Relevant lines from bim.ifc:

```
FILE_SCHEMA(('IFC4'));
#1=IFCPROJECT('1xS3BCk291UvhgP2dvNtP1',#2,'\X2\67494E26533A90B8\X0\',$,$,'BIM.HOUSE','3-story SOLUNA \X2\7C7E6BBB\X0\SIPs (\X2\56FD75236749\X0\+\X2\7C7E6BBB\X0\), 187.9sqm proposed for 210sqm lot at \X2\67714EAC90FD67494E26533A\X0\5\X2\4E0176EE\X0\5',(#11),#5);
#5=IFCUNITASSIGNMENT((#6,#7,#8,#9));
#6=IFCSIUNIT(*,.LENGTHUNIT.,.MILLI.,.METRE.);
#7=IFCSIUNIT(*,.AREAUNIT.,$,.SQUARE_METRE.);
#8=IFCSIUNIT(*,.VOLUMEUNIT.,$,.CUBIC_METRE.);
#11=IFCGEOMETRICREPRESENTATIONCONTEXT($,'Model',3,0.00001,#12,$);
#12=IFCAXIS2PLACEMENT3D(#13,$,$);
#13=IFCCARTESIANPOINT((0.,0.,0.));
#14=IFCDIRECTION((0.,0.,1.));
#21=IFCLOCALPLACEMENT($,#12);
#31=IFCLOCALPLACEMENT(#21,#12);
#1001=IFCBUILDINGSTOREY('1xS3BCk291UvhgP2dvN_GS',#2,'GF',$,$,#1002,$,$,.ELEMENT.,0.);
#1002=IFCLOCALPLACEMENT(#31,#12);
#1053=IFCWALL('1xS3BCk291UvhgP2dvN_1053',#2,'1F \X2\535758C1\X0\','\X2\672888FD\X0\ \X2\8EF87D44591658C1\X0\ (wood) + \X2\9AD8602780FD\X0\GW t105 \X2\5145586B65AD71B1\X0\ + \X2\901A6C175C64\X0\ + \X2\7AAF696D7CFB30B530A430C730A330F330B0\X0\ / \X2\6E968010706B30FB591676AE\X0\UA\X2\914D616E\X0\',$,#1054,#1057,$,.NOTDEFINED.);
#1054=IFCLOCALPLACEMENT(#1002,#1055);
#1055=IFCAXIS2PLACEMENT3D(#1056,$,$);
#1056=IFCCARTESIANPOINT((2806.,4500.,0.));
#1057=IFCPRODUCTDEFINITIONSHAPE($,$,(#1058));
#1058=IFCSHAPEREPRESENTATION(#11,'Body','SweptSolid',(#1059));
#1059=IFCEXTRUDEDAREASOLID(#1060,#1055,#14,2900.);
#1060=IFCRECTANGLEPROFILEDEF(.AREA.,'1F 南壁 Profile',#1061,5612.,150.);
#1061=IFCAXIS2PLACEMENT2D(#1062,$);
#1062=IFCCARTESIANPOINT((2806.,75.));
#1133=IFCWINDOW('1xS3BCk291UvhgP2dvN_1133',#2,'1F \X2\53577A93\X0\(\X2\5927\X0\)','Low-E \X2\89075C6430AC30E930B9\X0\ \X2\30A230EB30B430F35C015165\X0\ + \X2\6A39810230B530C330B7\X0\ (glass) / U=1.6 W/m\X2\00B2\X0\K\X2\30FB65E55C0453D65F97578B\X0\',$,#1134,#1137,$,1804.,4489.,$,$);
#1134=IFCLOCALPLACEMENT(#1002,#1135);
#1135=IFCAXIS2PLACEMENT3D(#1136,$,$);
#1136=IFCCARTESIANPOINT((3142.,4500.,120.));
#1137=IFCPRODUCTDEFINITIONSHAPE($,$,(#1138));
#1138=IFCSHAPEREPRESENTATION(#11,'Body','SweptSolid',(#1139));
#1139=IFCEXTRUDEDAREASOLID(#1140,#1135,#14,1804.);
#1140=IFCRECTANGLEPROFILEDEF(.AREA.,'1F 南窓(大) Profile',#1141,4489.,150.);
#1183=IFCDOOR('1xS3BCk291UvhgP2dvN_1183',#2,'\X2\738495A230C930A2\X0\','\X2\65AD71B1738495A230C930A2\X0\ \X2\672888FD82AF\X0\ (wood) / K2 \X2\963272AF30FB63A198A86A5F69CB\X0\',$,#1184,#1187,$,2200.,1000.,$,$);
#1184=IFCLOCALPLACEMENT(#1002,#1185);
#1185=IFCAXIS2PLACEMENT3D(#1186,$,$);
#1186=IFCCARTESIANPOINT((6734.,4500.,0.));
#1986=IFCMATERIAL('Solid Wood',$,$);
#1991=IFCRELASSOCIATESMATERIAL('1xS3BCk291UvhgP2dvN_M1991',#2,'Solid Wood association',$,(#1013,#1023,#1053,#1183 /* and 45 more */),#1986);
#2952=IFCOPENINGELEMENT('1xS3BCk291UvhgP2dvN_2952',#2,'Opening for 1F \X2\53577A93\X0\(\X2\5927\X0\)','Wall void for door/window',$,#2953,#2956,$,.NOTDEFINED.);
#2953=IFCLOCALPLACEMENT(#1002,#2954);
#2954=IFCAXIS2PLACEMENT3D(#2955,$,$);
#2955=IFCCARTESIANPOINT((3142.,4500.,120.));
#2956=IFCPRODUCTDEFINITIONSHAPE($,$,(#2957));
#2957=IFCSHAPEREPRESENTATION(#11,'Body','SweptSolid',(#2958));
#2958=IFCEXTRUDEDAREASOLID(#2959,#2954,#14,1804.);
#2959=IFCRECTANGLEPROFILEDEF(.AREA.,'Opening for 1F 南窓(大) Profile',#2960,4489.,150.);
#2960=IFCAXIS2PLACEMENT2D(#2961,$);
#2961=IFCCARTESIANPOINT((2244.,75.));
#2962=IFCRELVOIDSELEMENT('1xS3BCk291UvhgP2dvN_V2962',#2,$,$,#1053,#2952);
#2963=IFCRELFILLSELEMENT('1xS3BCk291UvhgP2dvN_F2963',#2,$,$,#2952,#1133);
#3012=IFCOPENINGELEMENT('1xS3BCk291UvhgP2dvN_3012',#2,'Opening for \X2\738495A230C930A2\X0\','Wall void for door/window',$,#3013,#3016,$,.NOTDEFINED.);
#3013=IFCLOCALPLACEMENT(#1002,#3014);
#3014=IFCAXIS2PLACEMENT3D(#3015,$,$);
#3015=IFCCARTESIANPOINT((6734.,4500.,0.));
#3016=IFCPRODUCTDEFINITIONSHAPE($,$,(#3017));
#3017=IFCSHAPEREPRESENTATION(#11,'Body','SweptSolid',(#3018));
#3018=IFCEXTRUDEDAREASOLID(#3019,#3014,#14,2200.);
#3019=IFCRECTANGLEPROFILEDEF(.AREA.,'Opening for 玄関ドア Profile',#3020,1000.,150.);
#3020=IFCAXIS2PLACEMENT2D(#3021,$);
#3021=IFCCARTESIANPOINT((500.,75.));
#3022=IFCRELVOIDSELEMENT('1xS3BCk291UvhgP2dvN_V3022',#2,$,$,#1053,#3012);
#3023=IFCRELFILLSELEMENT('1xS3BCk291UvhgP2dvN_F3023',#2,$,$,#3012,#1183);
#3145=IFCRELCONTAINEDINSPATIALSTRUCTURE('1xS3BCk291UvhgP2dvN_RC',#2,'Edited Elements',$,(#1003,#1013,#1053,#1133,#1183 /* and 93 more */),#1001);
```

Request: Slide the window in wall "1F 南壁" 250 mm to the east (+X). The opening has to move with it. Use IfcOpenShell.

```python
import ifcopenshell
import ifcopenshell.api.geometry
import ifcopenshell.util.placement

model = ifcopenshell.open("bim.ifc")

window = model.by_guid("1xS3BCk291UvhgP2dvN_1133")
opening = window.FillsVoids[0].RelatingOpeningElement
wall = opening.VoidsElements[0].RelatingBuildingElement

wall_matrix = ifcopenshell.util.placement.get_local_placement(wall.ObjectPlacement)
shift = wall_matrix[:3, 0] * 250.0
before = ifcopenshell.util.placement.get_local_placement(window.ObjectPlacement)[:3, 3].copy()

# The window is not placed relative to its opening, so move both.
for product in (opening, window):
    matrix = ifcopenshell.util.placement.get_local_placement(product.ObjectPlacement)
    matrix[:3, 3] += shift
    ifcopenshell.api.geometry.edit_object_placement(model, product=product, matrix=matrix, is_si=False)

after = ifcopenshell.util.placement.get_local_placement(window.ObjectPlacement)[:3, 3]
print("window moved by", (after - before).round(3) + 0.0)

model.write("bim_rev.ifc")
```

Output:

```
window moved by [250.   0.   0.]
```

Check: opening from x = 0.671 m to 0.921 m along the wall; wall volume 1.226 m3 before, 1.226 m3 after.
